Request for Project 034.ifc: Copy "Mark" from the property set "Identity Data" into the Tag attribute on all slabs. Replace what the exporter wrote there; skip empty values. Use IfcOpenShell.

First a look at what the model holds.

```python
import ifcopenshell
import ifcopenshell.util.element

model = ifcopenshell.open("Project 034.ifc")
print(model.schema)
slabs = model.by_type("IfcSlab")
print(len(slabs), "slabs")
for e in slabs[:8]:
    source = ifcopenshell.util.element.get_pset(e, "Identity Data", "Mark")
    target = e.Tag
    print(e.id(), repr(source), repr(target), sep=" | ")
```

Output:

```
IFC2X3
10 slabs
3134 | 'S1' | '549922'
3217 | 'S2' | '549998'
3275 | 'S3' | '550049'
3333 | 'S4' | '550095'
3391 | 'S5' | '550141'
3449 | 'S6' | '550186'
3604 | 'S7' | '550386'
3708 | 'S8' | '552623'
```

```python
import ifcopenshell
import ifcopenshell.util.element

model = ifcopenshell.open("Project 034.ifc")

count = 0
for e in model.by_type("IfcSlab"):
    value = ifcopenshell.util.element.get_pset(e, "Identity Data", "Mark")
    current = e.Tag
    if not value or not value.strip() or current == value:
        continue
    e.Tag = value
    count += 1

print(count, "slabs updated")

model.write("Project 034-out.ifc")
```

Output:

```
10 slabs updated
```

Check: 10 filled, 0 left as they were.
